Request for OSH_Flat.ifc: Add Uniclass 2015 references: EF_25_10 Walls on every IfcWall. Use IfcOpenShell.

First a look at what the model holds.

```python
import ifcopenshell

model = ifcopenshell.open("OSH_Flat.ifc")
print(model.schema)
print("classifications:", [c.Name for c in model.by_type("IfcClassification")])
for ifc_class in ("IfcDoor", "IfcRoof", "IfcStair", "IfcWall", "IfcWindow"):
    print(ifc_class, len(model.by_type(ifc_class)))
```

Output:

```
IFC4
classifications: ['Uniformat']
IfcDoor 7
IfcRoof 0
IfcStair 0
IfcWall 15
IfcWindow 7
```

```python
import ifcopenshell
import ifcopenshell.api.classification

model = ifcopenshell.open("OSH_Flat.ifc")

system = ifcopenshell.api.classification.add_classification(model, classification="Uniclass 2015")

codes = {
    "IfcWall": ("EF_25_10", "Walls"),
}
for ifc_class, (code, name) in codes.items():
    products = model.by_type(ifc_class)
    ifcopenshell.api.classification.add_reference(
        model, products=products, classification=system, identification=code, name=name
    )
    print(code, len(products))

model.write("OSH_Flat_edited.ifc")
```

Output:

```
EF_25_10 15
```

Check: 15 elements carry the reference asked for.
